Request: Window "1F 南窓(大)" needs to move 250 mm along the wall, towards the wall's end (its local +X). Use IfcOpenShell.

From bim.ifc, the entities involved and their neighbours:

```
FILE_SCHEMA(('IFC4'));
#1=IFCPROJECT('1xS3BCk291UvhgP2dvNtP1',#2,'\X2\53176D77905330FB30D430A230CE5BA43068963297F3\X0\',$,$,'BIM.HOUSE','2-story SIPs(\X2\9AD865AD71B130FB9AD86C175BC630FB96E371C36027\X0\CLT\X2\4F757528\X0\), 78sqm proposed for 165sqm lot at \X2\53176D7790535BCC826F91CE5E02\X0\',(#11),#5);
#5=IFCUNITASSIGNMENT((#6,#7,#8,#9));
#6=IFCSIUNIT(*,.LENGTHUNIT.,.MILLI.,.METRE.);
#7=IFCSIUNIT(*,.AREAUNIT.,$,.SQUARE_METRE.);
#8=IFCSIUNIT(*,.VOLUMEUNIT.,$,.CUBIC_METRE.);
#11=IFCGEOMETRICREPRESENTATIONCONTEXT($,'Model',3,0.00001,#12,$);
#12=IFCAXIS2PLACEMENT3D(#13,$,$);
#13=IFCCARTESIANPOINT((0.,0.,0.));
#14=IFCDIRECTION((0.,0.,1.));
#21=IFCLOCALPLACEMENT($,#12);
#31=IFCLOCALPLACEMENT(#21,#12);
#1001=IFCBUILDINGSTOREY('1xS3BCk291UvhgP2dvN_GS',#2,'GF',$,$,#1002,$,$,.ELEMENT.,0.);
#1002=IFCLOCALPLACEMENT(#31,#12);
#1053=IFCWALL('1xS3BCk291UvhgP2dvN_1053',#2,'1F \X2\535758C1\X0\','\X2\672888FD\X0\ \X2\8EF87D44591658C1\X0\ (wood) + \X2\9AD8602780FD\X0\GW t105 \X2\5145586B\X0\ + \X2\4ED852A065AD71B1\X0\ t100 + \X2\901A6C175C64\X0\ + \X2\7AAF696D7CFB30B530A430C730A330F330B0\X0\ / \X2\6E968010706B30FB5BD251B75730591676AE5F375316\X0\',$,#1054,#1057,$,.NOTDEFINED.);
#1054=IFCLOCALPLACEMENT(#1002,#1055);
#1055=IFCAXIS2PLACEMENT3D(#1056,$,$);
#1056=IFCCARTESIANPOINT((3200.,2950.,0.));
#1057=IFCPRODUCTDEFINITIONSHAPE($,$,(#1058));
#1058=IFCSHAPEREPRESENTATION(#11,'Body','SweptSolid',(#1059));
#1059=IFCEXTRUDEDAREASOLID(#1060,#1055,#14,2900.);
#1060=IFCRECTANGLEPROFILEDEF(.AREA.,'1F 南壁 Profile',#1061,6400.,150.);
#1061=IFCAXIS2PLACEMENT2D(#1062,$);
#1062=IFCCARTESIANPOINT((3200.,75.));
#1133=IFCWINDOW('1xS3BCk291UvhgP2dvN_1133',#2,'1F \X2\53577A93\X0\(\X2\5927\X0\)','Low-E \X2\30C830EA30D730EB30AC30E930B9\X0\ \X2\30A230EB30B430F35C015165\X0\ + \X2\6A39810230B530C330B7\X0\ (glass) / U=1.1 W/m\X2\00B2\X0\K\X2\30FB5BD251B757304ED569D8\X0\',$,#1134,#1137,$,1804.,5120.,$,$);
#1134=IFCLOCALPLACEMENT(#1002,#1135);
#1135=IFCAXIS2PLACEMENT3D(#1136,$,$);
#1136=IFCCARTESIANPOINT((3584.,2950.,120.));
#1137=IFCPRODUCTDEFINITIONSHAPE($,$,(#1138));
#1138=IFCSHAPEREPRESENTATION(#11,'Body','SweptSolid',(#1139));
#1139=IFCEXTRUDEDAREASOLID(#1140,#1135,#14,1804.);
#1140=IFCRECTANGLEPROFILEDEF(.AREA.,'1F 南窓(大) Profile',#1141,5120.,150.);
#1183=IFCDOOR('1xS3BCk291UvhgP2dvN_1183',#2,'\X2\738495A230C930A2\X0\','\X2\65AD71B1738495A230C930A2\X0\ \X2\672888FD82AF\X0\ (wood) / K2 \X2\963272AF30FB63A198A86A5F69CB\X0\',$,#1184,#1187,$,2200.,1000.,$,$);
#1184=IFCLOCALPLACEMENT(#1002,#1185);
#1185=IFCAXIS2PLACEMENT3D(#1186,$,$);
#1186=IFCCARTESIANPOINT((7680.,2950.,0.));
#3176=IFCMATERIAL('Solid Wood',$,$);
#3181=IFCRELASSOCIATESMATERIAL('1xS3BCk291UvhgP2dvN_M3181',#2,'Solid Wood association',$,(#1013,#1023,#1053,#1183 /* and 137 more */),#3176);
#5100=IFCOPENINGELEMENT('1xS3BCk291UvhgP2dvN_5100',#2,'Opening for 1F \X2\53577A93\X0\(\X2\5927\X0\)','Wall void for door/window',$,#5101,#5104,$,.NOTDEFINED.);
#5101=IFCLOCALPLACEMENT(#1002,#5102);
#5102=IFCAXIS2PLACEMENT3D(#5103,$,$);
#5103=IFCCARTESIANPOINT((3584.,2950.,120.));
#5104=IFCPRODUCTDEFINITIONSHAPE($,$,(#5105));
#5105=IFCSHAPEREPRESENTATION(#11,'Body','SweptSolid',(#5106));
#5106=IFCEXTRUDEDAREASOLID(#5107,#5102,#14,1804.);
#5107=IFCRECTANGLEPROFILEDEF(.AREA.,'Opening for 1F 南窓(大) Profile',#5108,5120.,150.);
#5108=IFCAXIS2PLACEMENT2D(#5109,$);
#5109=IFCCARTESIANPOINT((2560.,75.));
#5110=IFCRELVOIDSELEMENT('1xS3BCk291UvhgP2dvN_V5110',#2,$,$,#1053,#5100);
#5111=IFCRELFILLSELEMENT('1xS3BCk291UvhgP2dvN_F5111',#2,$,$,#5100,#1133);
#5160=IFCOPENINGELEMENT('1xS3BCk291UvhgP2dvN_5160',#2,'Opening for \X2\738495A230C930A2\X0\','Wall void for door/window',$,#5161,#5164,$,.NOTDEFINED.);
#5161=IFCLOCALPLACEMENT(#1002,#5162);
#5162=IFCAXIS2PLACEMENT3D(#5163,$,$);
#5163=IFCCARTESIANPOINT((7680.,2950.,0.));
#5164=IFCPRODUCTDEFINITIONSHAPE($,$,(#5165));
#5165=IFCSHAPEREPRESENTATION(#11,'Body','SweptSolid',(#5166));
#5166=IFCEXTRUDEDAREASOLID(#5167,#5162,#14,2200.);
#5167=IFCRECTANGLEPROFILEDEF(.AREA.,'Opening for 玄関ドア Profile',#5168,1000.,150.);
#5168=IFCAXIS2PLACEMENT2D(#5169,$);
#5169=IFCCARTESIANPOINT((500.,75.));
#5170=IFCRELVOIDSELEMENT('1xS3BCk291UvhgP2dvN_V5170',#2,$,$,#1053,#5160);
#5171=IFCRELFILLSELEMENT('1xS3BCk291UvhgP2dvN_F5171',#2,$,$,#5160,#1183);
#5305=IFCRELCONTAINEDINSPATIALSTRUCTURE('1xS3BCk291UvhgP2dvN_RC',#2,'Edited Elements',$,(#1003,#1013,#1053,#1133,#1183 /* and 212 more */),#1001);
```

```python
import ifcopenshell
import ifcopenshell.api.geometry
import ifcopenshell.util.placement

model = ifcopenshell.open("bim.ifc")

window = model.by_id(1133)
opening = window.FillsVoids[0].RelatingOpeningElement
wall = opening.VoidsElements[0].RelatingBuildingElement

wall_matrix = ifcopenshell.util.placement.get_local_placement(wall.ObjectPlacement)
shift = wall_matrix[:3, 0] * 250.0
before = ifcopenshell.util.placement.get_local_placement(window.ObjectPlacement)[:3, 3].copy()

# The window is not placed relative to its opening, so move both.
for product in (opening, window):
    matrix = ifcopenshell.util.placement.get_local_placement(product.ObjectPlacement)
    matrix[:3, 3] += shift
    ifcopenshell.api.geometry.edit_object_placement(model, product=product, matrix=matrix, is_si=False)

after = ifcopenshell.util.placement.get_local_placement(window.ObjectPlacement)[:3, 3]
print("window moved by", (after - before).round(3) + 0.0)

model.write("bim_rev.ifc")
```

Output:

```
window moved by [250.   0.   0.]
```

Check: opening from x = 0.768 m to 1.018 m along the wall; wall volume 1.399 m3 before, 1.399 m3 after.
